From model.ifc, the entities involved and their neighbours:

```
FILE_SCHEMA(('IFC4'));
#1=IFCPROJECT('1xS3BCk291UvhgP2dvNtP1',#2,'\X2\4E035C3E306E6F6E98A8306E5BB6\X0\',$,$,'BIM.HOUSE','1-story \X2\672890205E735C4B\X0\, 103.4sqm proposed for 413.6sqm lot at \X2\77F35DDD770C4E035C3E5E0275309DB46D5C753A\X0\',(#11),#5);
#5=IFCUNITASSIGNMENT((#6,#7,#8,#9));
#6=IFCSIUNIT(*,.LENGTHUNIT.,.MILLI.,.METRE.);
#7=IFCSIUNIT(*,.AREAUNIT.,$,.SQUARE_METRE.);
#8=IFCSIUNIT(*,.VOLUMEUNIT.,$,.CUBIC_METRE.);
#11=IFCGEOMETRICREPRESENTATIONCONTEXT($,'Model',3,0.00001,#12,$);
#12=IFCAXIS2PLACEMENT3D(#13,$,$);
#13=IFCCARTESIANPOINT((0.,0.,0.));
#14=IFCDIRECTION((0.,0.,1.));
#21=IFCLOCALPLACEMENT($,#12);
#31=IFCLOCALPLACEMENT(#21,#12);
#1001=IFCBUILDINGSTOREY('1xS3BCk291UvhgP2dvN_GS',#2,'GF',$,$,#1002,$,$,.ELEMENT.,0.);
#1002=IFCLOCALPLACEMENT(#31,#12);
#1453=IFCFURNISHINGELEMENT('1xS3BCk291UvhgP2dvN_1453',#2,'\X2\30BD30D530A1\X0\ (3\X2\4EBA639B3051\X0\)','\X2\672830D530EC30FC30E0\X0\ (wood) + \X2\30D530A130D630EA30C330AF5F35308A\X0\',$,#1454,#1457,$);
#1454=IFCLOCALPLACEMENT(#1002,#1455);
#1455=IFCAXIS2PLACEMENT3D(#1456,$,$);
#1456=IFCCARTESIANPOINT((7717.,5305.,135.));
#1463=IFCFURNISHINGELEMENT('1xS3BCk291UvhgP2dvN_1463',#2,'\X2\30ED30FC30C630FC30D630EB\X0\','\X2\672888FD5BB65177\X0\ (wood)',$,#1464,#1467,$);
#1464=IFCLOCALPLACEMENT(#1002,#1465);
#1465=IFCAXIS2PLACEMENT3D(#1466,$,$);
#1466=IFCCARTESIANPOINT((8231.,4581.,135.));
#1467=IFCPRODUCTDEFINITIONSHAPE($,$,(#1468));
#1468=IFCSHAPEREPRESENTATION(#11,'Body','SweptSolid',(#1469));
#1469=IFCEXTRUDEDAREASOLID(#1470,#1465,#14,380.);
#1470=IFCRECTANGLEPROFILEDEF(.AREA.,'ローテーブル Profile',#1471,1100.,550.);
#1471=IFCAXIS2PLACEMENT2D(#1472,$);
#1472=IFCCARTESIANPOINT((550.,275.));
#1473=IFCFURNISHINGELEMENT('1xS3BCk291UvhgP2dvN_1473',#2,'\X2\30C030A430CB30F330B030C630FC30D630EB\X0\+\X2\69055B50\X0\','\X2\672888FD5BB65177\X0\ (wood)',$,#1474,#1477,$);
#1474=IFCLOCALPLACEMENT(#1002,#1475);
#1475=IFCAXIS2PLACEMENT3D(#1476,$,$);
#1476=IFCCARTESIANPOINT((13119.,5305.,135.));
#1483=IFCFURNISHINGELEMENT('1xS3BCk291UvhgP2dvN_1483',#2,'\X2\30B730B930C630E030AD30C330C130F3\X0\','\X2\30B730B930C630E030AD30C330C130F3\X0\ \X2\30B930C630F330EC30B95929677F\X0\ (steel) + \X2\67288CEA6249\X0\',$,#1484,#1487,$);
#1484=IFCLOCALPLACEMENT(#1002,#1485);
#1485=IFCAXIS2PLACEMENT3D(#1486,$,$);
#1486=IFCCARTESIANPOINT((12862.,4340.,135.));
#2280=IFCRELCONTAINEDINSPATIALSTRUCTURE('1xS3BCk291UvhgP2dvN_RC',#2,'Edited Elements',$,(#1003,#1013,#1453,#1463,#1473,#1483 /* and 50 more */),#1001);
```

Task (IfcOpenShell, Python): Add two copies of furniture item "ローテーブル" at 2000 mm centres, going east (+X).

```python
import numpy as np
import ifcopenshell
import ifcopenshell.api.geometry
import ifcopenshell.api.root
import ifcopenshell.util.element
import ifcopenshell.util.placement
import ifcopenshell.util.unit

model = ifcopenshell.open("model.ifc")
unit_scale = ifcopenshell.util.unit.calculate_unit_scale(model)


def reuse_history(source, copy):
    """copy_class also copies each property set's owner history, people and application; keep the originals."""
    for rel in copy.IsDefinedBy:
        if rel.is_a("IfcRelDefinesByProperties") and (history := rel.RelatingPropertyDefinition.OwnerHistory):
            rel.RelatingPropertyDefinition.OwnerHistory = source.OwnerHistory
            ifcopenshell.util.element.remove_deep2(model, history)


source = model.by_guid("1xS3BCk291UvhgP2dvN_1463")
base = ifcopenshell.util.placement.get_local_placement(source.ObjectPlacement)
step = np.array([1.0, 0.0, 0.0]) * 2 / unit_scale

for i in range(1, 3):
    copy = ifcopenshell.api.root.copy_class(model, product=source)
    copy.Representation = ifcopenshell.util.element.copy_deep(
        model, source.Representation, exclude=["IfcGeometricRepresentationContext", "IfcRepresentationMap"]
    )
    reuse_history(source, copy)
    matrix = base.copy()
    matrix[:3, 3] += i * step
    print("added at", matrix[:3, 3].round(3) + 0.0)
    ifcopenshell.api.geometry.edit_object_placement(model, product=copy, matrix=matrix, is_si=False)

model.write("model_v2.ifc")
```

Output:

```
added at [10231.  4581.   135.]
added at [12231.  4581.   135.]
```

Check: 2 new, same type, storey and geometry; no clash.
